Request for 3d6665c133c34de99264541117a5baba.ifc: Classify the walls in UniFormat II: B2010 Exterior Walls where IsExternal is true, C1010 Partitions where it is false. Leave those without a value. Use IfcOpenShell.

First a look at what the model holds.

```python
import ifcopenshell
import ifcopenshell.util.element

model = ifcopenshell.open("3d6665c133c34de99264541117a5baba.ifc")
print(model.schema)
print("classifications:", [c.Name for c in model.by_type("IfcClassification")])
values = [ifcopenshell.util.element.get_pset(e, "Pset_WallCommon", "IsExternal") for e in model.by_type("IfcWall")]
for value in (True, False, None):
    print("IsExternal", value, values.count(value))
```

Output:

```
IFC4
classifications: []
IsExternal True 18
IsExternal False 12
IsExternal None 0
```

```python
import ifcopenshell
import ifcopenshell.api.classification
import ifcopenshell.util.element

model = ifcopenshell.open("3d6665c133c34de99264541117a5baba.ifc")

system = ifcopenshell.api.classification.add_classification(model, classification="UniFormat II")

walls = model.by_type("IfcWall")
external = {e: ifcopenshell.util.element.get_pset(e, "Pset_WallCommon", "IsExternal") for e in walls}
for flag, code, name in ((True, "B2010", "Exterior Walls"), (False, "C1010", "Partitions")):
    products = [e for e in walls if external[e] is flag]
    ifcopenshell.api.classification.add_reference(
        model, products=products, classification=system, identification=code, name=name
    )
    print(code, len(products))

model.write("3d6665c133c34de99264541117a5baba_updated.ifc")
```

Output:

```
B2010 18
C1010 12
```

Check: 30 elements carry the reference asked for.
